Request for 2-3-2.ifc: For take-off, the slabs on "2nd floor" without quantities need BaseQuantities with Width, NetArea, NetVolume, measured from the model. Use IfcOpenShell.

First a look at what the model holds.

```python
import ifcopenshell
import ifcopenshell.util.element
import ifcopenshell.util.unit

model = ifcopenshell.open("2-3-2.ifc")
print(model.schema)
for unit_type in ("LENGTHUNIT", "AREAUNIT", "VOLUMEUNIT"):
    print(unit_type, ifcopenshell.util.unit.calculate_unit_scale(model, unit_type))
storey = next(s for s in model.by_type("IfcBuildingStorey") if s.Name == "2nd floor")
slabs = [e for e in ifcopenshell.util.element.get_decomposition(storey) if e.is_a("IfcSlab")]
for e in sorted(slabs, key=lambda e: e.id()):
    print(e.id(), e.is_a(), e.Name, list(ifcopenshell.util.element.get_psets(e, qtos_only=True)), sep=" | ")
```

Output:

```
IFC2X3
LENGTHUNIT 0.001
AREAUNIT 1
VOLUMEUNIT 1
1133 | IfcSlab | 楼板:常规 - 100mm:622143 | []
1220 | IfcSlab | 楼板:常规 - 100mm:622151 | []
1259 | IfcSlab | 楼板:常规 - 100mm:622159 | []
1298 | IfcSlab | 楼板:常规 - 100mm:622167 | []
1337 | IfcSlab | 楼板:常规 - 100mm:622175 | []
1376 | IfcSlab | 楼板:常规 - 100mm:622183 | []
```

```python
import ifcopenshell
import ifcopenshell.api.pset
import ifcopenshell.geom
import ifcopenshell.util.element
import ifcopenshell.util.shape
import ifcopenshell.util.unit

model = ifcopenshell.open("2-3-2.ifc")
unit_scale = ifcopenshell.util.unit.calculate_unit_scale(model)
area_scale = ifcopenshell.util.unit.calculate_unit_scale(model, "AREAUNIT")
volume_scale = ifcopenshell.util.unit.calculate_unit_scale(model, "VOLUMEUNIT")
settings = ifcopenshell.geom.settings()

storey = next(s for s in model.by_type("IfcBuildingStorey") if s.Name == "2nd floor")
slabs = [e for e in ifcopenshell.util.element.get_decomposition(storey) if e.is_a("IfcSlab")]

for e in sorted(slabs, key=lambda e: e.id()):
    if ifcopenshell.util.element.get_psets(e, qtos_only=True, should_inherit=False):
        continue
    # Geometry comes back in metres, in the element's own axes.
    shape = ifcopenshell.geom.create_shape(settings, e)
    values = {
        "Width": ifcopenshell.util.shape.get_z(shape.geometry) / unit_scale,
        "NetArea": ifcopenshell.util.shape.get_footprint_area(shape.geometry) / area_scale,
        "NetVolume": ifcopenshell.util.shape.get_volume(shape.geometry) / volume_scale,
    }
    qto = ifcopenshell.api.pset.add_qto(model, product=e, name="BaseQuantities")
    ifcopenshell.api.pset.edit_qto(model, qto=qto, properties=values)
    print(e.id(), {k: round(v, 3) for k, v in values.items()})

model.write("2-3-2-out.ifc")
```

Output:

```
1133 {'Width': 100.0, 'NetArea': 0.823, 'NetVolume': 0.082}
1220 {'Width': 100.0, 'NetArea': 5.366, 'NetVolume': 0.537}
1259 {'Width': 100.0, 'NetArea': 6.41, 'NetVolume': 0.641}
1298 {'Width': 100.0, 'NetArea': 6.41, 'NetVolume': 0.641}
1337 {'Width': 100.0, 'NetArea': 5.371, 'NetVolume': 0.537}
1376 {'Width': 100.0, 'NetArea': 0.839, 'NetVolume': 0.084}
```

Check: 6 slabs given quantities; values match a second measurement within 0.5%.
